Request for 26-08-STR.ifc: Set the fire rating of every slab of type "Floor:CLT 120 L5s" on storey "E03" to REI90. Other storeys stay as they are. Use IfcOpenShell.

First a look at what the model holds.

```python
import ifcopenshell
import ifcopenshell.util.element

model = ifcopenshell.open("26-08-STR.ifc")
print(model.schema)
storey = next(s for s in model.by_type("IfcBuildingStorey") if s.Name == "E03")
slabs = [e for e in ifcopenshell.util.element.get_decomposition(storey) if e.is_a("IfcSlab")]
seen = {}
for e in slabs:
    element_type = ifcopenshell.util.element.get_type(e)
    key = (element_type.Name if element_type != e and element_type else None, ifcopenshell.util.element.get_pset(e, "Pset_SlabCommon", "FireRating"))
    seen[key] = seen.get(key, 0) + 1
for (name, value), count in sorted(seen.items(), key=str):
    print(count, "x", name, "|", value)
```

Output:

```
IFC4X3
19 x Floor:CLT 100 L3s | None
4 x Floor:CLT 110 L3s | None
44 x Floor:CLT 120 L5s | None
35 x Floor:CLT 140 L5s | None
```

```python
import ifcopenshell
import ifcopenshell.api.pset
import ifcopenshell.util.element

model = ifcopenshell.open("26-08-STR.ifc")

storey = next(s for s in model.by_type("IfcBuildingStorey") if s.Name == "E03")
slabs = [e for e in ifcopenshell.util.element.get_decomposition(storey) if e.is_a("IfcSlab")]

count = 0
for e in slabs:
    element_type = ifcopenshell.util.element.get_type(e)
    if element_type in (None, e) or element_type.Name != "Floor:CLT 120 L5s":
        continue
    # add_pset returns the element's existing set when there is one.
    pset = ifcopenshell.api.pset.add_pset(model, product=e, name="Pset_SlabCommon")
    ifcopenshell.api.pset.edit_pset(model, pset=pset, properties={"FireRating": "REI90"})
    count += 1

print(count, "slabs updated")

model.write("26-08-STR_edited.ifc")
```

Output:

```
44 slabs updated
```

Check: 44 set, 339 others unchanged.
